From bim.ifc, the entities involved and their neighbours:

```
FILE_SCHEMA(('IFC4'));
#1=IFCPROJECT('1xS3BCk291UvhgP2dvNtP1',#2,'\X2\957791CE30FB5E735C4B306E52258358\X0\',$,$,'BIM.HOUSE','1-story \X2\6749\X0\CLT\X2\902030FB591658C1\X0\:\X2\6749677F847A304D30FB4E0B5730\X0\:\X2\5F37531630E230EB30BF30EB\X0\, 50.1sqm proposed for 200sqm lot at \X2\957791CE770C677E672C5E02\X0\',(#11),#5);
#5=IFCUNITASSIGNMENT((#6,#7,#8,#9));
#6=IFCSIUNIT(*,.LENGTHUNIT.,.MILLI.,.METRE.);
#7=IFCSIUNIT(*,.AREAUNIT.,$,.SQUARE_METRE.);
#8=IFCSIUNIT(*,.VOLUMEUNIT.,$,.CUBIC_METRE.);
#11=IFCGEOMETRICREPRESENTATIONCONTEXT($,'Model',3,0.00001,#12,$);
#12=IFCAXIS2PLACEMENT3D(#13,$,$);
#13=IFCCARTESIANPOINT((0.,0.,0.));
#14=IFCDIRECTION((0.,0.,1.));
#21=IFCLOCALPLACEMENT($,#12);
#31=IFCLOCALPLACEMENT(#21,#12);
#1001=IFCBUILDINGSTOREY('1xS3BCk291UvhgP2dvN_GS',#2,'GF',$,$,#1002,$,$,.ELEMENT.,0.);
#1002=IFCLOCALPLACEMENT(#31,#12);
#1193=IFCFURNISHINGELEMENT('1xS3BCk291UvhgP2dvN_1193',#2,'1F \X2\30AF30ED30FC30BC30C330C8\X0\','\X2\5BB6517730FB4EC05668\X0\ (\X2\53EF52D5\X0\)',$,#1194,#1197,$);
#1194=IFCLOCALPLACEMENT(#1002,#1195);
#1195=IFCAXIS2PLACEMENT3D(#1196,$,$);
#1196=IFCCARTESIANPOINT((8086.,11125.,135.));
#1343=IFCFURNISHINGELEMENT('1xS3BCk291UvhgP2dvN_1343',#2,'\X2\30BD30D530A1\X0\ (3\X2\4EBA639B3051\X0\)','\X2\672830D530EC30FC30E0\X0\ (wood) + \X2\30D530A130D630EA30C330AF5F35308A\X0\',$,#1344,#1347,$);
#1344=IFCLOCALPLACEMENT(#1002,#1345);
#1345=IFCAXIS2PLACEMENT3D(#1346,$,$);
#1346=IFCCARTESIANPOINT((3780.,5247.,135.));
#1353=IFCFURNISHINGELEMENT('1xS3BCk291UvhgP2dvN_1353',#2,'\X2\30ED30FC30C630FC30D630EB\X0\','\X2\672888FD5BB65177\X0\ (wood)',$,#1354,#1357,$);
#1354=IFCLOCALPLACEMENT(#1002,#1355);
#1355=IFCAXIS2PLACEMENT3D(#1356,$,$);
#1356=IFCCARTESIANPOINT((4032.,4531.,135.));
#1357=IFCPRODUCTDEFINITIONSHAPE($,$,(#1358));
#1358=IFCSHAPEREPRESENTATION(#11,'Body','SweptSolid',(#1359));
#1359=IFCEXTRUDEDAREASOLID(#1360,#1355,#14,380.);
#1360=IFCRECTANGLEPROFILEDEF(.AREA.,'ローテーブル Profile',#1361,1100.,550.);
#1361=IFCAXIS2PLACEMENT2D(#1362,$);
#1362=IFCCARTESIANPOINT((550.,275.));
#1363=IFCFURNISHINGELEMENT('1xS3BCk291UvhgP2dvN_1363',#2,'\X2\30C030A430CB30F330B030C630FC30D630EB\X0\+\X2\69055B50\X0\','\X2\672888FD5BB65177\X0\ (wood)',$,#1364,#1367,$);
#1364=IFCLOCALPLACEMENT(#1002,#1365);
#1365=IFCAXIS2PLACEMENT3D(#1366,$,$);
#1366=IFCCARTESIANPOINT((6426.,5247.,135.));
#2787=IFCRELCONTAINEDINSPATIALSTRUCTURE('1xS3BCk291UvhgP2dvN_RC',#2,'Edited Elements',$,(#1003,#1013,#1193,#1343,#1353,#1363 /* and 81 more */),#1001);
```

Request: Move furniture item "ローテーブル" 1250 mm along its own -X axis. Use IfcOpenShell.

```python
import ifcopenshell
import ifcopenshell.api.geometry
import ifcopenshell.util.placement
import ifcopenshell.util.unit

model = ifcopenshell.open("bim.ifc")
unit_scale = ifcopenshell.util.unit.calculate_unit_scale(model)

item = model.by_guid("1xS3BCk291UvhgP2dvN_1353")
matrix = ifcopenshell.util.placement.get_local_placement(item.ObjectPlacement)
matrix[:3, 3] -= matrix[:3, 0] * 1.25 / unit_scale
ifcopenshell.api.geometry.edit_object_placement(model, product=item, matrix=matrix, is_si=False)

print(ifcopenshell.util.placement.get_local_placement(item.ObjectPlacement).round(3) + 0.0)

model.write("bim_rev.ifc")
```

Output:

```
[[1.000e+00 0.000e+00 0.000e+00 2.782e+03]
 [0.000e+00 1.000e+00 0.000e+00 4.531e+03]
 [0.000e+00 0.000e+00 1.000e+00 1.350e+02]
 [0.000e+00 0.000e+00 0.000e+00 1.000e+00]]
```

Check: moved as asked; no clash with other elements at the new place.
